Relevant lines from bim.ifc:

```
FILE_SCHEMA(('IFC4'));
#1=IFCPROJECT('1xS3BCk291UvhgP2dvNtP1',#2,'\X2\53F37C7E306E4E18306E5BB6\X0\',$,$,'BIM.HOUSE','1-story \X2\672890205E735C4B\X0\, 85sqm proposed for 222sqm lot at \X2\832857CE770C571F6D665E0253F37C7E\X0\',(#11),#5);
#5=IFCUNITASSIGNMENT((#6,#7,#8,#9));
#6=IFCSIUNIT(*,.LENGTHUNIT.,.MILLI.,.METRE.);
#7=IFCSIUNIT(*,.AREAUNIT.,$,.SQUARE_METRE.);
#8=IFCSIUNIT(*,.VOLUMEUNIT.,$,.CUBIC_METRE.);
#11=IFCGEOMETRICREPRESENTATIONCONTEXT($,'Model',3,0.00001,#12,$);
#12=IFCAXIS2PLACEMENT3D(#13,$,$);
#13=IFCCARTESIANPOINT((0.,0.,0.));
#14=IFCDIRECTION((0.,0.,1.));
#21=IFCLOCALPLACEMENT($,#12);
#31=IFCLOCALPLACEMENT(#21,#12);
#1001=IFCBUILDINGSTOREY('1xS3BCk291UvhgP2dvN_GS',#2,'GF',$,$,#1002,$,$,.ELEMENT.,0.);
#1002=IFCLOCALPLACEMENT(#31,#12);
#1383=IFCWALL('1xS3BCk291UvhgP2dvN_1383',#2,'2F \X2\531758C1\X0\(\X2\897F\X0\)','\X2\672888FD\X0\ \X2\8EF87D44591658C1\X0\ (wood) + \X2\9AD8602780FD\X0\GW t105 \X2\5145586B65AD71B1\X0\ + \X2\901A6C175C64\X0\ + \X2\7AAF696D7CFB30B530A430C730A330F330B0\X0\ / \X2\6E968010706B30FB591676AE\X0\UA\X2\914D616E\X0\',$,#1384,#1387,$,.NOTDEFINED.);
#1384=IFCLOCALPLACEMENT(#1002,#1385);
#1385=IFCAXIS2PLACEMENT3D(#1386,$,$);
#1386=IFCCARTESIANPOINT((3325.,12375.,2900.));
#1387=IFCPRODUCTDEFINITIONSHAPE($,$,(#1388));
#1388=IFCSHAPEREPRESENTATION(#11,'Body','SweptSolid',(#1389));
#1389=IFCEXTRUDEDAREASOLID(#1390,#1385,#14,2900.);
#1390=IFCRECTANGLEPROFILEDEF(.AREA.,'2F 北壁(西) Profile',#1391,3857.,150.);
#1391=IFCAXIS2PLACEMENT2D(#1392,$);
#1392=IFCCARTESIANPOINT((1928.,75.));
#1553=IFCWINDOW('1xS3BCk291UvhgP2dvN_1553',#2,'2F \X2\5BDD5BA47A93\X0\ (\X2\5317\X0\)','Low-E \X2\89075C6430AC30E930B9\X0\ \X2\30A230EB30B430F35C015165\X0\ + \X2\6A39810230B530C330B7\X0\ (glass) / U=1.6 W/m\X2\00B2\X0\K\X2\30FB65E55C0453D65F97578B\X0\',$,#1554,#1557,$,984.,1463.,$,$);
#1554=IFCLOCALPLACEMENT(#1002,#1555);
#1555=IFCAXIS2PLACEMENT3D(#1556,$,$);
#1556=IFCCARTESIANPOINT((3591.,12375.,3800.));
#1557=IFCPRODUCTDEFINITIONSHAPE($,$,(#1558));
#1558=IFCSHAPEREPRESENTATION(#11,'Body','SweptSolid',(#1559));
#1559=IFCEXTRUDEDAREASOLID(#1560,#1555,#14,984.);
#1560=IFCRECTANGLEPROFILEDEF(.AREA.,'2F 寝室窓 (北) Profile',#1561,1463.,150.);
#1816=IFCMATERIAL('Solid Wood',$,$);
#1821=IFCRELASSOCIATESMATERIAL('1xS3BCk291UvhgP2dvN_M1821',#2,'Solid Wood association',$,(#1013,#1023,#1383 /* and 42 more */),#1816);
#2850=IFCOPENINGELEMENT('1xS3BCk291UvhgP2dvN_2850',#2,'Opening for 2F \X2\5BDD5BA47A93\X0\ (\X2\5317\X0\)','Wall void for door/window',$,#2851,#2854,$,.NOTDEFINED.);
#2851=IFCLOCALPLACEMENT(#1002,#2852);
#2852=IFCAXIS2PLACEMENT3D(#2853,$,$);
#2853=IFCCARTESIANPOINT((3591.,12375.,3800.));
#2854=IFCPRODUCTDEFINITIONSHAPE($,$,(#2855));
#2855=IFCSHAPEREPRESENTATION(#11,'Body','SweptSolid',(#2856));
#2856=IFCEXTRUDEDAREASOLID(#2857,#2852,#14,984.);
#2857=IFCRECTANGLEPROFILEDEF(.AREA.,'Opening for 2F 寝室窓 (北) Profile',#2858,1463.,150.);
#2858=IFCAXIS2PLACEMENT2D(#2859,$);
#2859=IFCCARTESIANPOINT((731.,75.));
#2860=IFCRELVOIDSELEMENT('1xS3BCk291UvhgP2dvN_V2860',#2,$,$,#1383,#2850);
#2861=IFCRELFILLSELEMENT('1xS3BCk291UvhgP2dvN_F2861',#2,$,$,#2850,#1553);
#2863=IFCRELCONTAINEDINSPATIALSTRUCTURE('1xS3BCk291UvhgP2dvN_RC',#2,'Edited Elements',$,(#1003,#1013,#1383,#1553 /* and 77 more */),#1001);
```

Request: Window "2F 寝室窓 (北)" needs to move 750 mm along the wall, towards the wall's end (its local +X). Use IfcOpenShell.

```python
import ifcopenshell
import ifcopenshell.api.geometry
import ifcopenshell.util.placement
import ifcopenshell.util.unit

model = ifcopenshell.open("bim.ifc")
unit_scale = ifcopenshell.util.unit.calculate_unit_scale(model)

window = model.by_guid("1xS3BCk291UvhgP2dvN_1553")
opening = window.FillsVoids[0].RelatingOpeningElement
wall = opening.VoidsElements[0].RelatingBuildingElement

wall_matrix = ifcopenshell.util.placement.get_local_placement(wall.ObjectPlacement)
shift = wall_matrix[:3, 0] * 0.75 / unit_scale
before = ifcopenshell.util.placement.get_local_placement(window.ObjectPlacement)[:3, 3].copy()

# The window is not placed relative to its opening, so move both.
for product in (opening, window):
    matrix = ifcopenshell.util.placement.get_local_placement(product.ObjectPlacement)
    matrix[:3, 3] += shift
    ifcopenshell.api.geometry.edit_object_placement(model, product=product, matrix=matrix, is_si=False)

after = ifcopenshell.util.placement.get_local_placement(window.ObjectPlacement)[:3, 3]
print("window moved by", (after - before).round(3) + 0.0)

model.write("bim_edited.ifc")
```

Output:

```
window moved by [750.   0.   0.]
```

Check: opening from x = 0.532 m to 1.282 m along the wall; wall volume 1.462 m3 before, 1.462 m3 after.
